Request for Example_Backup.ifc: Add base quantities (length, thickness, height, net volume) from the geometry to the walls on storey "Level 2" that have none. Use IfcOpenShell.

First a look at what the model holds.

```python
import ifcopenshell
import ifcopenshell.util.element
import ifcopenshell.util.unit

model = ifcopenshell.open("Example_Backup.ifc")
print(model.schema)
for unit_type in ("LENGTHUNIT", "AREAUNIT", "VOLUMEUNIT"):
    print(unit_type, ifcopenshell.util.unit.calculate_unit_scale(model, unit_type))
storey = next(s for s in model.by_type("IfcBuildingStorey") if s.Name == "Level 2")
walls = [e for e in ifcopenshell.util.element.get_decomposition(storey) if e.is_a("IfcWall")]
for e in sorted(walls, key=lambda e: e.id()):
    print(e.id(), e.is_a(), e.Name, list(ifcopenshell.util.element.get_psets(e, qtos_only=True)), sep=" | ")
```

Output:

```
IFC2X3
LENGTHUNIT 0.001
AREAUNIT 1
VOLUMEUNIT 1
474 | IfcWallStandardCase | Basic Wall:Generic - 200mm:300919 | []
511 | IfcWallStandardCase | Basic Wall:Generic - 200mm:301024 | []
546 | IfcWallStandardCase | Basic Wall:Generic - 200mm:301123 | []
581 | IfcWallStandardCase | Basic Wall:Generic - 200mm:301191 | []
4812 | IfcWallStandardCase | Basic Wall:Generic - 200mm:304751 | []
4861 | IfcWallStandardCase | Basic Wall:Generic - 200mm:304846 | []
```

```python
import ifcopenshell
import ifcopenshell.api.pset
import ifcopenshell.geom
import ifcopenshell.util.element
import ifcopenshell.util.shape
import ifcopenshell.util.unit

model = ifcopenshell.open("Example_Backup.ifc")
unit_scale = ifcopenshell.util.unit.calculate_unit_scale(model)
volume_scale = ifcopenshell.util.unit.calculate_unit_scale(model, "VOLUMEUNIT")
settings = ifcopenshell.geom.settings()

storey = next(s for s in model.by_type("IfcBuildingStorey") if s.Name == "Level 2")
walls = [e for e in ifcopenshell.util.element.get_decomposition(storey) if e.is_a("IfcWall")]

for e in sorted(walls, key=lambda e: e.id()):
    if ifcopenshell.util.element.get_psets(e, qtos_only=True, should_inherit=False):
        continue
    # Geometry comes back in metres, in the element's own axes.
    shape = ifcopenshell.geom.create_shape(settings, e)
    values = {
        "Length": ifcopenshell.util.shape.get_x(shape.geometry) / unit_scale,
        "Width": ifcopenshell.util.shape.get_y(shape.geometry) / unit_scale,
        "Height": ifcopenshell.util.shape.get_z(shape.geometry) / unit_scale,
        "NetVolume": ifcopenshell.util.shape.get_volume(shape.geometry) / volume_scale,
    }
    qto = ifcopenshell.api.pset.add_qto(model, product=e, name="BaseQuantities")
    ifcopenshell.api.pset.edit_qto(model, qto=qto, properties=values)
    print(e.id(), {k: round(v, 3) for k, v in values.items()})

model.write("Example_Backup_edited.ifc")
```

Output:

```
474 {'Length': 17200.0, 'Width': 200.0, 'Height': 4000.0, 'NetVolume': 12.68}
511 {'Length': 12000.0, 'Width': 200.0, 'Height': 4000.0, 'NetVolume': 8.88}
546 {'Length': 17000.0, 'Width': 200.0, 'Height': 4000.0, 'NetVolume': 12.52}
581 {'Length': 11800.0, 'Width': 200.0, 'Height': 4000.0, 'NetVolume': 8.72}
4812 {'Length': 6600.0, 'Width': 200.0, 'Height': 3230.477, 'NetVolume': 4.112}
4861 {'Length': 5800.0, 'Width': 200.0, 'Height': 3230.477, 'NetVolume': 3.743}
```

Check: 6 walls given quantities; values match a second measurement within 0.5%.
